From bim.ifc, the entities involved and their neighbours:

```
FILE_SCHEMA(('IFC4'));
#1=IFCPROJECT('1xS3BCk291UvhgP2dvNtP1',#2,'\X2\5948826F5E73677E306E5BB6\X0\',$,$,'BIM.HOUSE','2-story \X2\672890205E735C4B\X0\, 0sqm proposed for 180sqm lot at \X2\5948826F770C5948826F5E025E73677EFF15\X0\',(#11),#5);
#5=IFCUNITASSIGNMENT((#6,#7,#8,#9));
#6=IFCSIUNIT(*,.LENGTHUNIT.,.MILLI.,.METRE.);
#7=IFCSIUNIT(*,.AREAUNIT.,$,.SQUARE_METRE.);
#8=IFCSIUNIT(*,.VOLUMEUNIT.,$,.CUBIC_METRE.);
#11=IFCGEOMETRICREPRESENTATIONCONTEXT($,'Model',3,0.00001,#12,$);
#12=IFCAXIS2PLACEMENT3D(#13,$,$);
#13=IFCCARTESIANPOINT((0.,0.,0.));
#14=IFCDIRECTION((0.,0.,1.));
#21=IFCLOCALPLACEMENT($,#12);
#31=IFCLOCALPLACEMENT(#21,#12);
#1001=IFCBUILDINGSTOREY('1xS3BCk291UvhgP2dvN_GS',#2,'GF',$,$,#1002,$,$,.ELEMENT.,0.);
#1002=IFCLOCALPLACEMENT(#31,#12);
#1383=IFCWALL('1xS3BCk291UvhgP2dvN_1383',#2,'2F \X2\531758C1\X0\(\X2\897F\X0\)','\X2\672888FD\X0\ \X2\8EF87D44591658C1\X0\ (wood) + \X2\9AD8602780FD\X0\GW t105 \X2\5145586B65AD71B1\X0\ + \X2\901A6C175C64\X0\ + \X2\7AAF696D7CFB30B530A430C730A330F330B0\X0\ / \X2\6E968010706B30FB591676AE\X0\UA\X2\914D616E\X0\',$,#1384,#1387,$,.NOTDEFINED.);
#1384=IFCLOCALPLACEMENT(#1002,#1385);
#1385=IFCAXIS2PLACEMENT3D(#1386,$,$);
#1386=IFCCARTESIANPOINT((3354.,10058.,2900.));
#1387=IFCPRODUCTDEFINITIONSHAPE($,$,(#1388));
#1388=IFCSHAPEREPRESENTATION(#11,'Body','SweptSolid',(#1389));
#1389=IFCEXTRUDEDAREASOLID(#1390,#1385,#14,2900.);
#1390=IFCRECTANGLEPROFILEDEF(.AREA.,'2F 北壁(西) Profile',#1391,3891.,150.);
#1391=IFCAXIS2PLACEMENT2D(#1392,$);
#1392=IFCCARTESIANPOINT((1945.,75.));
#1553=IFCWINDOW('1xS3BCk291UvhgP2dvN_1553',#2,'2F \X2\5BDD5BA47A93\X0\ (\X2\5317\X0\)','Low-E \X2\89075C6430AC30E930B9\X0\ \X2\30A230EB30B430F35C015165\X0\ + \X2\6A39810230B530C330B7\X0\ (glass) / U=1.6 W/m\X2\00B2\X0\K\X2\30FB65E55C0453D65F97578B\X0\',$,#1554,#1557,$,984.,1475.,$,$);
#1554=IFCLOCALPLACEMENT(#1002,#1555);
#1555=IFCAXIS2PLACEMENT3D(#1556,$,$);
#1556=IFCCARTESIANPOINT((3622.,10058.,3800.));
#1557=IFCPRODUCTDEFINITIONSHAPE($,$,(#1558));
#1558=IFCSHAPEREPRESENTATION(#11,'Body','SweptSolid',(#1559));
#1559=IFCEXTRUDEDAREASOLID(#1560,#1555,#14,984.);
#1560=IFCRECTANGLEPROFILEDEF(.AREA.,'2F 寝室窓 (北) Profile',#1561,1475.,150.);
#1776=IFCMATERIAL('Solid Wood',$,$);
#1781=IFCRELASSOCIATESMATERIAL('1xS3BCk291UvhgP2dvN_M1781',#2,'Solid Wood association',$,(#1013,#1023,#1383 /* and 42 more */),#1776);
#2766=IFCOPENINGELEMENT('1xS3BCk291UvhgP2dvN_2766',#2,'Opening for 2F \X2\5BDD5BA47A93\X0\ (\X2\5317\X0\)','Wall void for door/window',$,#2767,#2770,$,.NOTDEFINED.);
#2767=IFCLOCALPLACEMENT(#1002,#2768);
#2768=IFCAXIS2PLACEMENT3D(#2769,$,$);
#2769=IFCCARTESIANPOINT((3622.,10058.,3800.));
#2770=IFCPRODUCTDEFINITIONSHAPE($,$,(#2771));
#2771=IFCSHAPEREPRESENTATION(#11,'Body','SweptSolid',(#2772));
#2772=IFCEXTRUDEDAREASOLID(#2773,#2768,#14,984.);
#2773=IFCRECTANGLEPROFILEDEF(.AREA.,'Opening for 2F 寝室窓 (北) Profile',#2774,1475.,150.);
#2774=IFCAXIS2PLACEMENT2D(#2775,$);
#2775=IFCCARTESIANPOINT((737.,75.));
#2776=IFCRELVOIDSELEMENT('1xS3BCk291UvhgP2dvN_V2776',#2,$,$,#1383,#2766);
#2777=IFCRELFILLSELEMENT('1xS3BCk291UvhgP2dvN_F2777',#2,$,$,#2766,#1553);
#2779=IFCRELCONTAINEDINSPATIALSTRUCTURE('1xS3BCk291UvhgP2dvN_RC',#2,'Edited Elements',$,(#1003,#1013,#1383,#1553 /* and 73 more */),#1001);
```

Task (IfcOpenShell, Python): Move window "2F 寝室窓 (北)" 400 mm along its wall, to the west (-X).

```python
import ifcopenshell
import ifcopenshell.api.geometry
import ifcopenshell.util.placement

model = ifcopenshell.open("bim.ifc")

window = model.by_guid("1xS3BCk291UvhgP2dvN_1553")
opening = window.FillsVoids[0].RelatingOpeningElement
wall = opening.VoidsElements[0].RelatingBuildingElement

wall_matrix = ifcopenshell.util.placement.get_local_placement(wall.ObjectPlacement)
shift = wall_matrix[:3, 0] * -400.0
before = ifcopenshell.util.placement.get_local_placement(window.ObjectPlacement)[:3, 3].copy()

# The window is not placed relative to its opening, so move both.
for product in (opening, window):
    matrix = ifcopenshell.util.placement.get_local_placement(product.ObjectPlacement)
    matrix[:3, 3] += shift
    ifcopenshell.api.geometry.edit_object_placement(model, product=product, matrix=matrix, is_si=False)

after = ifcopenshell.util.placement.get_local_placement(window.ObjectPlacement)[:3, 3]
print("window moved by", (after - before).round(3) + 0.0)

model.write("bim-out.ifc")
```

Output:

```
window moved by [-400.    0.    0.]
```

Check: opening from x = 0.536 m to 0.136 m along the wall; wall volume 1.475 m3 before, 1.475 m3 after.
